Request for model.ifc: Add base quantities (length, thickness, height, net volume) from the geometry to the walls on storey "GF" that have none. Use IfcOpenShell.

First a look at what the model holds.

```python
import ifcopenshell
import ifcopenshell.util.element
import ifcopenshell.util.unit

model = ifcopenshell.open("model.ifc")
print(model.schema)
for unit_type in ("LENGTHUNIT", "AREAUNIT", "VOLUMEUNIT"):
    print(unit_type, ifcopenshell.util.unit.calculate_unit_scale(model, unit_type))
storey = next(s for s in model.by_type("IfcBuildingStorey") if s.Name == "GF")
walls = [e for e in ifcopenshell.util.element.get_decomposition(storey) if e.is_a("IfcWall")]
for e in sorted(walls, key=lambda e: e.id()):
    print(e.id(), e.is_a(), e.Name, list(ifcopenshell.util.element.get_psets(e, qtos_only=True)), sep=" | ")
```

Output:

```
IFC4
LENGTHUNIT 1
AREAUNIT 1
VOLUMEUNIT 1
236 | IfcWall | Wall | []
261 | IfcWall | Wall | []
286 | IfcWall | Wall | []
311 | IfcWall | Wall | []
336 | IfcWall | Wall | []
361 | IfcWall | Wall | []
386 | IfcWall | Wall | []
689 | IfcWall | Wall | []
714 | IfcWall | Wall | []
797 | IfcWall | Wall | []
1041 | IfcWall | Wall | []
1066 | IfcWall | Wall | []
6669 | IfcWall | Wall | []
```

```python
import ifcopenshell
import ifcopenshell.api.pset
import ifcopenshell.geom
import ifcopenshell.util.element
import ifcopenshell.util.shape
import ifcopenshell.util.unit

model = ifcopenshell.open("model.ifc")
unit_scale = ifcopenshell.util.unit.calculate_unit_scale(model)
volume_scale = ifcopenshell.util.unit.calculate_unit_scale(model, "VOLUMEUNIT")
settings = ifcopenshell.geom.settings()

storey = next(s for s in model.by_type("IfcBuildingStorey") if s.Name == "GF")
walls = [e for e in ifcopenshell.util.element.get_decomposition(storey) if e.is_a("IfcWall")]

for e in sorted(walls, key=lambda e: e.id()):
    if ifcopenshell.util.element.get_psets(e, qtos_only=True, should_inherit=False):
        continue
    # Geometry comes back in metres, in the element's own axes.
    shape = ifcopenshell.geom.create_shape(settings, e)
    values = {
        "Length": ifcopenshell.util.shape.get_x(shape.geometry) / unit_scale,
        "Width": ifcopenshell.util.shape.get_y(shape.geometry) / unit_scale,
        "Height": ifcopenshell.util.shape.get_z(shape.geometry) / unit_scale,
        "NetVolume": ifcopenshell.util.shape.get_volume(shape.geometry) / volume_scale,
    }
    qto = ifcopenshell.api.pset.add_qto(model, product=e, name="Qto_WallBaseQuantities")
    ifcopenshell.api.pset.edit_qto(model, qto=qto, properties=values)
    print(e.id(), {k: round(v, 3) for k, v in values.items()})

model.write("model_v2.ifc")
```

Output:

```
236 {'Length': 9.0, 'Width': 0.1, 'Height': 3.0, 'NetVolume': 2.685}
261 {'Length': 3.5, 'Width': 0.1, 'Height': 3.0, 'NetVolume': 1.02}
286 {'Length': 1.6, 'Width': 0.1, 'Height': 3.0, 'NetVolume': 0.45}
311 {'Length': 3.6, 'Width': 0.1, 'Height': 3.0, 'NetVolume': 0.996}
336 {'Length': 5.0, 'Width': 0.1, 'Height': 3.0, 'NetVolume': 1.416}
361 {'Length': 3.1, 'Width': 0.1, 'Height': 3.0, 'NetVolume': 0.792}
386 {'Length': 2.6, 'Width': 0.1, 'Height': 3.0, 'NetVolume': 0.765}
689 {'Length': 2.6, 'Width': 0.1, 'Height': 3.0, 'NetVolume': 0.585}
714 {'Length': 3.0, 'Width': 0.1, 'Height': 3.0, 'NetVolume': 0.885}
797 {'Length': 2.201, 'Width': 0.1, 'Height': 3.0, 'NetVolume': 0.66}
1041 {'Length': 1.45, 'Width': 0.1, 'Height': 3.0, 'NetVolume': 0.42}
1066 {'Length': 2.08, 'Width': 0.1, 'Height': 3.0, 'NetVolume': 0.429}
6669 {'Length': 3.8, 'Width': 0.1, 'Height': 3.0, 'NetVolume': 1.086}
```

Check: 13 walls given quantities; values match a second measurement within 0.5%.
